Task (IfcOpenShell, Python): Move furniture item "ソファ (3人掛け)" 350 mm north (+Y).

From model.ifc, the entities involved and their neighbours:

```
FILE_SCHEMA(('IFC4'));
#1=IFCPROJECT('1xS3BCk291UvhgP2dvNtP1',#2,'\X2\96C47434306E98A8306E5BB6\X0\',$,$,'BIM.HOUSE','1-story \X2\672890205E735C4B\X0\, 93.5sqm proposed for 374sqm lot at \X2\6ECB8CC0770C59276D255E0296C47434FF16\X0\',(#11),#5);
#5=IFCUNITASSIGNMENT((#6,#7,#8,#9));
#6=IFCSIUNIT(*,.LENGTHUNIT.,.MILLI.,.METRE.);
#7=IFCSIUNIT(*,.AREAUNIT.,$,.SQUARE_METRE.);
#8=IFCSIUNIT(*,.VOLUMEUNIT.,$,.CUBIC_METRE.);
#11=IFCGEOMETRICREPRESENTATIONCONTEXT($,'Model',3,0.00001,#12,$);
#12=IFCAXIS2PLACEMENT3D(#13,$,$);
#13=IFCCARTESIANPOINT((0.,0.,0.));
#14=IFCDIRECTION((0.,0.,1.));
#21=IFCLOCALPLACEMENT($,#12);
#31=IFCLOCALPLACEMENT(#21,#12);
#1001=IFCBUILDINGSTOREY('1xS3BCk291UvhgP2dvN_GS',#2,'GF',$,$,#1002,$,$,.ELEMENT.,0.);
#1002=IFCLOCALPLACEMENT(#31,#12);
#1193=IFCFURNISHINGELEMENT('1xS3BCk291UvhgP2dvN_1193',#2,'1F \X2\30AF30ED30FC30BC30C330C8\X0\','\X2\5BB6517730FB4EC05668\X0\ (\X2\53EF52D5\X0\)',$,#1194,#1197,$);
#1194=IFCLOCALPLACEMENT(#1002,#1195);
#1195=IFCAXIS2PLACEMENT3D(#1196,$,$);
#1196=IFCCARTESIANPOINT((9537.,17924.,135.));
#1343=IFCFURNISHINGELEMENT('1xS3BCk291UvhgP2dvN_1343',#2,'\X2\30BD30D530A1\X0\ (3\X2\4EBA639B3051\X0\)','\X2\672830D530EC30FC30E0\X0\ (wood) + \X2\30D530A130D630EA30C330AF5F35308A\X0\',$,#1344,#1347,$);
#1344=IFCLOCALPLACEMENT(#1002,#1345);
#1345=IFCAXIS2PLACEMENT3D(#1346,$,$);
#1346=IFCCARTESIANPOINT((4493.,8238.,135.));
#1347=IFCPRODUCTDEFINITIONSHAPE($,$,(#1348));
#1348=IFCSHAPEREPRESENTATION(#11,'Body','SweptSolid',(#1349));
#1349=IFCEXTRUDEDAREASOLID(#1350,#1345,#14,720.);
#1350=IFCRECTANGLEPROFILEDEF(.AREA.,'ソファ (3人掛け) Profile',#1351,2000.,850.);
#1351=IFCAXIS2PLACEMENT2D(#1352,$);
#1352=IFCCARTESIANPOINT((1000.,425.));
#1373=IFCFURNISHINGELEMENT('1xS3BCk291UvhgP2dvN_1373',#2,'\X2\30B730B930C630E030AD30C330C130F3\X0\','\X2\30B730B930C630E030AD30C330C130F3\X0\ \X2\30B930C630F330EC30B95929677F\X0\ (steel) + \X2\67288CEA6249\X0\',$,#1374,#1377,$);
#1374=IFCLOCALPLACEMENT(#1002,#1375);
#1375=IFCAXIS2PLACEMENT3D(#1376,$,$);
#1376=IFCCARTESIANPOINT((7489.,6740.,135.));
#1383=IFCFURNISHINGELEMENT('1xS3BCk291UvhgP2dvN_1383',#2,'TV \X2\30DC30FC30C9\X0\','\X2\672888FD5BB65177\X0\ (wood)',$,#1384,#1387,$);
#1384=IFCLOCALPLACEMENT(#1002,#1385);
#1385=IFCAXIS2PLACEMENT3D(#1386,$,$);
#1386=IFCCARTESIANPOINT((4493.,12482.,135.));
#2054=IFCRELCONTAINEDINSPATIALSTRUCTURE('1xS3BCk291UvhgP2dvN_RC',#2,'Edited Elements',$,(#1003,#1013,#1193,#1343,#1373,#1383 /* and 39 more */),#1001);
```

```python
import ifcopenshell
import ifcopenshell.api.geometry
import ifcopenshell.util.placement

model = ifcopenshell.open("model.ifc")

item = model.by_guid("1xS3BCk291UvhgP2dvN_1343")
matrix = ifcopenshell.util.placement.get_local_placement(item.ObjectPlacement)
matrix[1, 3] += 350.0
ifcopenshell.api.geometry.edit_object_placement(model, product=item, matrix=matrix, is_si=False)

print(ifcopenshell.util.placement.get_local_placement(item.ObjectPlacement).round(3) + 0.0)

model.write("model_updated.ifc")
```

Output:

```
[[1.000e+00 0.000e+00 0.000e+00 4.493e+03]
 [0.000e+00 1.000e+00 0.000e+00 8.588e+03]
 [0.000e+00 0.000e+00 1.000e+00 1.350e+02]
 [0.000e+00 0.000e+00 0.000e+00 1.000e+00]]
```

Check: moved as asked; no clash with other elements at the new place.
